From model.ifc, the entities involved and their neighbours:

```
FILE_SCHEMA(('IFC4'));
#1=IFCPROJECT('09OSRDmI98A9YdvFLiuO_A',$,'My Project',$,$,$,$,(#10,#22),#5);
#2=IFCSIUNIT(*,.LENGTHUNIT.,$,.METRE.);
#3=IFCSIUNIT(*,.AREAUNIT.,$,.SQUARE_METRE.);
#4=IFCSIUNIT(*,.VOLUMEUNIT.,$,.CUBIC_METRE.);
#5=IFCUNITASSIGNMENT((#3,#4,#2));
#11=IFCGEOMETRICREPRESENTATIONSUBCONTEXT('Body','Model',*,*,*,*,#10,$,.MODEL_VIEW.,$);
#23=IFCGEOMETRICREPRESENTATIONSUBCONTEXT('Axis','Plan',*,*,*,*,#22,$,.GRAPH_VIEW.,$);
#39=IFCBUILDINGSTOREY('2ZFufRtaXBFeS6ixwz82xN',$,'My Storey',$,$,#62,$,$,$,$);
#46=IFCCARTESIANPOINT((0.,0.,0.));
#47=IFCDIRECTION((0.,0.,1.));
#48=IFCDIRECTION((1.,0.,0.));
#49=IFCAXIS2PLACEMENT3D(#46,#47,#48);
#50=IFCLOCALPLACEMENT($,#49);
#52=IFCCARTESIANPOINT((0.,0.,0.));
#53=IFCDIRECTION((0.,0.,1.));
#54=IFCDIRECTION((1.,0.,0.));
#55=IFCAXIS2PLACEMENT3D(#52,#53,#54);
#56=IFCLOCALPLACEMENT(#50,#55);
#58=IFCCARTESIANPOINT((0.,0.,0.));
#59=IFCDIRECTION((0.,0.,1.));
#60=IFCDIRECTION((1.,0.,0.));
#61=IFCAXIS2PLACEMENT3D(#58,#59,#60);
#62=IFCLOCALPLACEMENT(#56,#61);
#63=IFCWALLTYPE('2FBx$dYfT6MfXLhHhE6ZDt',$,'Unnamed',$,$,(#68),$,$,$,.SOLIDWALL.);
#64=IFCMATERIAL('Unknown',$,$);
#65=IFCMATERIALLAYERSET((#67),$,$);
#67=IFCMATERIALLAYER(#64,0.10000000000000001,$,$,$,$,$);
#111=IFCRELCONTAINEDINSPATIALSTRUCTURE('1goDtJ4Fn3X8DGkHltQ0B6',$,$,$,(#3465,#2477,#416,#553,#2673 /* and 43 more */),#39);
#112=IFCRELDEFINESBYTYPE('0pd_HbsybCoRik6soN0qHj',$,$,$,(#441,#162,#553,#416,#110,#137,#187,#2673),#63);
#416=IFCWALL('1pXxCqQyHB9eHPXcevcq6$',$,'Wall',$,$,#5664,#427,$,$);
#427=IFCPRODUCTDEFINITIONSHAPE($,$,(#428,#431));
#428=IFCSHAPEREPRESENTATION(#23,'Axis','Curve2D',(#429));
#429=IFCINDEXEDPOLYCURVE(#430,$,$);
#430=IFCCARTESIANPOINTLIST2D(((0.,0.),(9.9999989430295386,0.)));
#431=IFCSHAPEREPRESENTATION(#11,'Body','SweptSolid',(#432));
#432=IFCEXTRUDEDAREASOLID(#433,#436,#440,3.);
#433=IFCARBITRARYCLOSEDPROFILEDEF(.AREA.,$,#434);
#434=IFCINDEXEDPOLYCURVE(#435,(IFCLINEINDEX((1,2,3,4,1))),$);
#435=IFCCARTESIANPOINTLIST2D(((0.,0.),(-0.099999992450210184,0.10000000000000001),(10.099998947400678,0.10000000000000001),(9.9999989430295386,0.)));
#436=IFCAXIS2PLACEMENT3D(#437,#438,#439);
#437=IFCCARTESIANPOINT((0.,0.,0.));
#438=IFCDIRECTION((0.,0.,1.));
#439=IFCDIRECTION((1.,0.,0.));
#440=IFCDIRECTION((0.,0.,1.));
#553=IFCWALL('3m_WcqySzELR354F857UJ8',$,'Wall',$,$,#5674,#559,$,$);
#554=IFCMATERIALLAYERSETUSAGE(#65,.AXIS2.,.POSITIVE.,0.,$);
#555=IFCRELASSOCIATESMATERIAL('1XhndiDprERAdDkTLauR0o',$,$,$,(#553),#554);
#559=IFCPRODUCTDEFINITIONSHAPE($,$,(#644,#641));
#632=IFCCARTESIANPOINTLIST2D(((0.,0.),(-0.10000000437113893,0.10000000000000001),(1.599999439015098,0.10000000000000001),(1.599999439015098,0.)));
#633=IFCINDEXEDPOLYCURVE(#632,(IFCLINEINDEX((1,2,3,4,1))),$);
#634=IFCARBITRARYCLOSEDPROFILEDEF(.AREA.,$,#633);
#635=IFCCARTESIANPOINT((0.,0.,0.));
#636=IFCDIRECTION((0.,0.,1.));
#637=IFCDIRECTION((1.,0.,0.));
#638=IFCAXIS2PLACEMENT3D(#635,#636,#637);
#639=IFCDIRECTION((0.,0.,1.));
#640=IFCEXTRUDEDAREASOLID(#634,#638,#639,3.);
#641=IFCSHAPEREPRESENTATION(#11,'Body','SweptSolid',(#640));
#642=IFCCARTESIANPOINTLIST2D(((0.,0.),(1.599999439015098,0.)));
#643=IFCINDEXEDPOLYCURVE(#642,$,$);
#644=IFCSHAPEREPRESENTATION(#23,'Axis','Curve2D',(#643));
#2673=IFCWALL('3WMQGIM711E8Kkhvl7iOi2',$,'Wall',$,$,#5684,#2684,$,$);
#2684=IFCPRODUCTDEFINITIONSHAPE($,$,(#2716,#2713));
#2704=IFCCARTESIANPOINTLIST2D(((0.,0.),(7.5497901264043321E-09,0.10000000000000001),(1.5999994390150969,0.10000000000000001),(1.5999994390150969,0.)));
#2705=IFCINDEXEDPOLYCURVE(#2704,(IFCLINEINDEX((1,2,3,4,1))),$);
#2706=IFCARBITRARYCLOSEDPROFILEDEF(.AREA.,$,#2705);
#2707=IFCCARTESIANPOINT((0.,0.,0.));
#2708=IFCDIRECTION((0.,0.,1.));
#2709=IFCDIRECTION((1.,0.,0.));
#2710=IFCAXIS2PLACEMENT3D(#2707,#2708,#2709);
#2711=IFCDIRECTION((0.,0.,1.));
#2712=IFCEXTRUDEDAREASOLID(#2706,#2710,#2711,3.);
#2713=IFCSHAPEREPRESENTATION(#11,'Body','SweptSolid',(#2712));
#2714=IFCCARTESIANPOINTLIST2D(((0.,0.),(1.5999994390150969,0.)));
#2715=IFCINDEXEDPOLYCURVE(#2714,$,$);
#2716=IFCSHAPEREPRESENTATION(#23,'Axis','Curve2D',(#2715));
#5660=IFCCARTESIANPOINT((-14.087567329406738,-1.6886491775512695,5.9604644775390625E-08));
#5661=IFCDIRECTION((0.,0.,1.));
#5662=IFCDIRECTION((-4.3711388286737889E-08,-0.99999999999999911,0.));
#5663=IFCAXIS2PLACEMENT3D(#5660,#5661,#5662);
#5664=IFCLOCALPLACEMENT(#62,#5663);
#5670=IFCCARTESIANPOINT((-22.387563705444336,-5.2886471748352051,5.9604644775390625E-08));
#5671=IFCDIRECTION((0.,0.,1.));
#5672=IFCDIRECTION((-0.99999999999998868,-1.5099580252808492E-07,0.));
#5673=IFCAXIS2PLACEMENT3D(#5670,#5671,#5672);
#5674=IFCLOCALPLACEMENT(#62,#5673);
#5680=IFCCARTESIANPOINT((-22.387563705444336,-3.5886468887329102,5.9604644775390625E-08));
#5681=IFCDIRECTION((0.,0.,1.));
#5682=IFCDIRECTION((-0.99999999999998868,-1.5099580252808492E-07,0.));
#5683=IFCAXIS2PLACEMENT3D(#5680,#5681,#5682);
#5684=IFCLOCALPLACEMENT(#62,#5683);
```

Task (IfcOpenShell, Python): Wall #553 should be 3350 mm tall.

```python
import ifcopenshell
import ifcopenshell.geom
import ifcopenshell.util.representation
import ifcopenshell.util.shape
import ifcopenshell.util.unit

model = ifcopenshell.open("model.ifc")
unit_scale = ifcopenshell.util.unit.calculate_unit_scale(model)
settings = ifcopenshell.geom.settings()


def volume(element):
    """Net volume in cubic metres, openings subtracted."""
    shape = ifcopenshell.geom.create_shape(settings, element)
    return ifcopenshell.util.shape.get_volume(shape.geometry)


wall = model.by_guid("3m_WcqySzELR354F857UJ8")
before = volume(wall)

body = ifcopenshell.util.representation.get_representation(wall, "Model", "Body")
solid = body.Items[0]
old_height = solid.Depth
solid.Depth = 3.35 / unit_scale
after = volume(wall)

print(f"height {old_height:g} -> {solid.Depth:g}, volume {before:.3f} -> {after:.3f} m3")

model.write("model_rev.ifc")
```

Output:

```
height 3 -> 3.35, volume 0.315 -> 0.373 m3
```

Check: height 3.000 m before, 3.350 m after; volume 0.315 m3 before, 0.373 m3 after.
